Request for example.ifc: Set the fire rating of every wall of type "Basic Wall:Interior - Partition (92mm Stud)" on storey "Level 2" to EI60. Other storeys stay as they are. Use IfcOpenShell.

First a look at what the model holds.

```python
import ifcopenshell
import ifcopenshell.util.element

model = ifcopenshell.open("example.ifc")
print(model.schema)
storey = next(s for s in model.by_type("IfcBuildingStorey") if s.Name == "Level 2")
walls = [e for e in ifcopenshell.util.element.get_decomposition(storey) if e.is_a("IfcWall")]
seen = {}
for e in walls:
    element_type = ifcopenshell.util.element.get_type(e)
    key = (element_type.Name if element_type != e and element_type else None, ifcopenshell.util.element.get_pset(e, "Pset_WallCommon", "FireRating"))
    seen[key] = seen.get(key, 0) + 1
for (name, value), count in sorted(seen.items(), key=str):
    print(count, "x", name, "|", value)
```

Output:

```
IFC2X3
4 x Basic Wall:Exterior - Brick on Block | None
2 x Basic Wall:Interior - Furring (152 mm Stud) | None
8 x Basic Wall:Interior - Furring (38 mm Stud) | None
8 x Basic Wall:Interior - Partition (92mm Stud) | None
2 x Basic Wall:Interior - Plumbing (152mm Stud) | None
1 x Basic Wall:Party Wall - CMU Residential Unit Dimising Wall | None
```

```python
import ifcopenshell
import ifcopenshell.api.pset
import ifcopenshell.util.element

model = ifcopenshell.open("example.ifc")

storey = next(s for s in model.by_type("IfcBuildingStorey") if s.Name == "Level 2")
walls = [e for e in ifcopenshell.util.element.get_decomposition(storey) if e.is_a("IfcWall")]

count = 0
for e in walls:
    element_type = ifcopenshell.util.element.get_type(e)
    if element_type in (None, e) or element_type.Name != "Basic Wall:Interior - Partition (92mm Stud)":
        continue
    # add_pset returns the element's existing set when there is one.
    pset = ifcopenshell.api.pset.add_pset(model, product=e, name="Pset_WallCommon")
    ifcopenshell.api.pset.edit_pset(model, pset=pset, properties={"FireRating": "EI60"})
    count += 1

print(count, "walls updated")

model.write("example_rev.ifc")
```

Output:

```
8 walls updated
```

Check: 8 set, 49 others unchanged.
